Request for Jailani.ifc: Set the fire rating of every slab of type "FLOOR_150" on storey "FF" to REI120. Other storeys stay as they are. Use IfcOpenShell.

First a look at what the model holds.

```python
import ifcopenshell
import ifcopenshell.util.element

model = ifcopenshell.open("Jailani.ifc")
print(model.schema)
storey = next(s for s in model.by_type("IfcBuildingStorey") if s.Name == "FF")
slabs = [e for e in ifcopenshell.util.element.get_decomposition(storey) if e.is_a("IfcSlab")]
seen = {}
for e in slabs:
    element_type = ifcopenshell.util.element.get_type(e)
    key = (element_type.Name if element_type != e and element_type else None, ifcopenshell.util.element.get_pset(e, "Pset_SlabCommon", "FireRating"))
    seen[key] = seen.get(key, 0) + 1
for (name, value), count in sorted(seen.items(), key=str):
    print(count, "x", name, "|", value)
```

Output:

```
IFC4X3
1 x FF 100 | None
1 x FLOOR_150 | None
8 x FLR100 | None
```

```python
import ifcopenshell
import ifcopenshell.api.pset
import ifcopenshell.util.element

model = ifcopenshell.open("Jailani.ifc")

storey = next(s for s in model.by_type("IfcBuildingStorey") if s.Name == "FF")
slabs = [e for e in ifcopenshell.util.element.get_decomposition(storey) if e.is_a("IfcSlab")]

count = 0
for e in slabs:
    element_type = ifcopenshell.util.element.get_type(e)
    if element_type in (None, e) or element_type.Name != "FLOOR_150":
        continue
    # add_pset returns the element's existing set when there is one.
    pset = ifcopenshell.api.pset.add_pset(model, product=e, name="Pset_SlabCommon")
    ifcopenshell.api.pset.edit_pset(model, pset=pset, properties={"FireRating": "REI120"})
    count += 1

print(count, "slabs updated")

model.write("Jailani_edited.ifc")
```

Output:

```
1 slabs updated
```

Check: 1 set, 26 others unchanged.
